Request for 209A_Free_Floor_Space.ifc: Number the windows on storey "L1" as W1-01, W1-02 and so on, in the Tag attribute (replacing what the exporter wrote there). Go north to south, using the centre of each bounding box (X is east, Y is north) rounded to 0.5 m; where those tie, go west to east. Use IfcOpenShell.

First a look at what the model holds.

```python
import ifcopenshell
import ifcopenshell.util.element
import ifcopenshell.util.placement

model = ifcopenshell.open("209A_Free_Floor_Space.ifc")
print(model.schema)
storey = next(s for s in model.by_type("IfcBuildingStorey") if s.Name == "L1")
windows = [e for e in ifcopenshell.util.element.get_decomposition(storey) if e.is_a("IfcWindow")]
for e in sorted(windows, key=lambda e: e.id()):
    origin = ifcopenshell.util.placement.get_local_placement(e.ObjectPlacement)[:3, 3]
    print(e.id(), e.Tag, e.Name, origin.round(2) + 0.0, sep=" | ")
```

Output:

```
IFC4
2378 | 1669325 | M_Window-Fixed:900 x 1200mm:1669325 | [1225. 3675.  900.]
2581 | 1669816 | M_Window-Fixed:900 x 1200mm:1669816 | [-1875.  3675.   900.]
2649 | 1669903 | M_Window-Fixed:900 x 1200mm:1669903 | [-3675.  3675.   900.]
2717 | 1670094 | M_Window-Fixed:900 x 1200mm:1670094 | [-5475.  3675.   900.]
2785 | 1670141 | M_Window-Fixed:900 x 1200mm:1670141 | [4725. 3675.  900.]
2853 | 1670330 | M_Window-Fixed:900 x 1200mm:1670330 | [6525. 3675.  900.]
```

```python
import ifcopenshell
import ifcopenshell.geom
import ifcopenshell.util.element
import ifcopenshell.util.shape

model = ifcopenshell.open("209A_Free_Floor_Space.ifc")
settings = ifcopenshell.geom.settings()
settings.set("use-world-coords", True)


def centre(element):
    shape = ifcopenshell.geom.create_shape(settings, element)
    return ifcopenshell.util.shape.get_bbox_centroid(shape.geometry)


storey = next(s for s in model.by_type("IfcBuildingStorey") if s.Name == "L1")
windows = [e for e in ifcopenshell.util.element.get_decomposition(storey) if e.is_a("IfcWindow")]

# Insertion points can sit at a corner or the storey origin, so sort by the geometry (in metres).
centres = {e: centre(e) for e in windows}
windows.sort(key=lambda e: (-round(centres[e][1] / 0.5), centres[e][0]))

for i, e in enumerate(windows, start=1):
    number = f"W1-{i:02d}"
    e.Tag = number
    print(e.id(), number)

model.write("209A_Free_Floor_Space_updated.ifc")
```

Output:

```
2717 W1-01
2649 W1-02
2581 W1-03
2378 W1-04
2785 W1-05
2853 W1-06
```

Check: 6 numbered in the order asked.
